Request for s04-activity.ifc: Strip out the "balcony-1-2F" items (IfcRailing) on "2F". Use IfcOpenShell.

First a look at what the model holds.

```python
import ifcopenshell
import ifcopenshell.util.element

model = ifcopenshell.open("s04-activity.ifc")
print(model.schema)
storey = next(s for s in model.by_type("IfcBuildingStorey") if s.Name == "2F")
railings = [e for e in ifcopenshell.util.element.get_decomposition(storey) if e.is_a("IfcRailing")]
seen = {}
for e in railings:
    element_type = ifcopenshell.util.element.get_type(e)
    name = element_type.Name if element_type not in (None, e) else None
    seen[name] = seen.get(name, 0) + 1
for name, count in sorted(seen.items(), key=str):
    print(count, "x", name)
```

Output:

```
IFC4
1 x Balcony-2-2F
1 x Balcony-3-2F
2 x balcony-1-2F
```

```python
import ifcopenshell
import ifcopenshell.api.root
import ifcopenshell.util.element

model = ifcopenshell.open("s04-activity.ifc")

storey = next(s for s in model.by_type("IfcBuildingStorey") if s.Name == "2F")
railings = [e for e in ifcopenshell.util.element.get_decomposition(storey) if e.is_a("IfcRailing")]
targets = [e for e in railings if (t := ifcopenshell.util.element.get_type(e)) not in (None, e) and t.Name == "balcony-1-2F"]

for e in targets:
    ifcopenshell.api.root.remove_product(model, product=e)
print(len(targets), "removed")

model.write("s04-activity_v2.ifc")
```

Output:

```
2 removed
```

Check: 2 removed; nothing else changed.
